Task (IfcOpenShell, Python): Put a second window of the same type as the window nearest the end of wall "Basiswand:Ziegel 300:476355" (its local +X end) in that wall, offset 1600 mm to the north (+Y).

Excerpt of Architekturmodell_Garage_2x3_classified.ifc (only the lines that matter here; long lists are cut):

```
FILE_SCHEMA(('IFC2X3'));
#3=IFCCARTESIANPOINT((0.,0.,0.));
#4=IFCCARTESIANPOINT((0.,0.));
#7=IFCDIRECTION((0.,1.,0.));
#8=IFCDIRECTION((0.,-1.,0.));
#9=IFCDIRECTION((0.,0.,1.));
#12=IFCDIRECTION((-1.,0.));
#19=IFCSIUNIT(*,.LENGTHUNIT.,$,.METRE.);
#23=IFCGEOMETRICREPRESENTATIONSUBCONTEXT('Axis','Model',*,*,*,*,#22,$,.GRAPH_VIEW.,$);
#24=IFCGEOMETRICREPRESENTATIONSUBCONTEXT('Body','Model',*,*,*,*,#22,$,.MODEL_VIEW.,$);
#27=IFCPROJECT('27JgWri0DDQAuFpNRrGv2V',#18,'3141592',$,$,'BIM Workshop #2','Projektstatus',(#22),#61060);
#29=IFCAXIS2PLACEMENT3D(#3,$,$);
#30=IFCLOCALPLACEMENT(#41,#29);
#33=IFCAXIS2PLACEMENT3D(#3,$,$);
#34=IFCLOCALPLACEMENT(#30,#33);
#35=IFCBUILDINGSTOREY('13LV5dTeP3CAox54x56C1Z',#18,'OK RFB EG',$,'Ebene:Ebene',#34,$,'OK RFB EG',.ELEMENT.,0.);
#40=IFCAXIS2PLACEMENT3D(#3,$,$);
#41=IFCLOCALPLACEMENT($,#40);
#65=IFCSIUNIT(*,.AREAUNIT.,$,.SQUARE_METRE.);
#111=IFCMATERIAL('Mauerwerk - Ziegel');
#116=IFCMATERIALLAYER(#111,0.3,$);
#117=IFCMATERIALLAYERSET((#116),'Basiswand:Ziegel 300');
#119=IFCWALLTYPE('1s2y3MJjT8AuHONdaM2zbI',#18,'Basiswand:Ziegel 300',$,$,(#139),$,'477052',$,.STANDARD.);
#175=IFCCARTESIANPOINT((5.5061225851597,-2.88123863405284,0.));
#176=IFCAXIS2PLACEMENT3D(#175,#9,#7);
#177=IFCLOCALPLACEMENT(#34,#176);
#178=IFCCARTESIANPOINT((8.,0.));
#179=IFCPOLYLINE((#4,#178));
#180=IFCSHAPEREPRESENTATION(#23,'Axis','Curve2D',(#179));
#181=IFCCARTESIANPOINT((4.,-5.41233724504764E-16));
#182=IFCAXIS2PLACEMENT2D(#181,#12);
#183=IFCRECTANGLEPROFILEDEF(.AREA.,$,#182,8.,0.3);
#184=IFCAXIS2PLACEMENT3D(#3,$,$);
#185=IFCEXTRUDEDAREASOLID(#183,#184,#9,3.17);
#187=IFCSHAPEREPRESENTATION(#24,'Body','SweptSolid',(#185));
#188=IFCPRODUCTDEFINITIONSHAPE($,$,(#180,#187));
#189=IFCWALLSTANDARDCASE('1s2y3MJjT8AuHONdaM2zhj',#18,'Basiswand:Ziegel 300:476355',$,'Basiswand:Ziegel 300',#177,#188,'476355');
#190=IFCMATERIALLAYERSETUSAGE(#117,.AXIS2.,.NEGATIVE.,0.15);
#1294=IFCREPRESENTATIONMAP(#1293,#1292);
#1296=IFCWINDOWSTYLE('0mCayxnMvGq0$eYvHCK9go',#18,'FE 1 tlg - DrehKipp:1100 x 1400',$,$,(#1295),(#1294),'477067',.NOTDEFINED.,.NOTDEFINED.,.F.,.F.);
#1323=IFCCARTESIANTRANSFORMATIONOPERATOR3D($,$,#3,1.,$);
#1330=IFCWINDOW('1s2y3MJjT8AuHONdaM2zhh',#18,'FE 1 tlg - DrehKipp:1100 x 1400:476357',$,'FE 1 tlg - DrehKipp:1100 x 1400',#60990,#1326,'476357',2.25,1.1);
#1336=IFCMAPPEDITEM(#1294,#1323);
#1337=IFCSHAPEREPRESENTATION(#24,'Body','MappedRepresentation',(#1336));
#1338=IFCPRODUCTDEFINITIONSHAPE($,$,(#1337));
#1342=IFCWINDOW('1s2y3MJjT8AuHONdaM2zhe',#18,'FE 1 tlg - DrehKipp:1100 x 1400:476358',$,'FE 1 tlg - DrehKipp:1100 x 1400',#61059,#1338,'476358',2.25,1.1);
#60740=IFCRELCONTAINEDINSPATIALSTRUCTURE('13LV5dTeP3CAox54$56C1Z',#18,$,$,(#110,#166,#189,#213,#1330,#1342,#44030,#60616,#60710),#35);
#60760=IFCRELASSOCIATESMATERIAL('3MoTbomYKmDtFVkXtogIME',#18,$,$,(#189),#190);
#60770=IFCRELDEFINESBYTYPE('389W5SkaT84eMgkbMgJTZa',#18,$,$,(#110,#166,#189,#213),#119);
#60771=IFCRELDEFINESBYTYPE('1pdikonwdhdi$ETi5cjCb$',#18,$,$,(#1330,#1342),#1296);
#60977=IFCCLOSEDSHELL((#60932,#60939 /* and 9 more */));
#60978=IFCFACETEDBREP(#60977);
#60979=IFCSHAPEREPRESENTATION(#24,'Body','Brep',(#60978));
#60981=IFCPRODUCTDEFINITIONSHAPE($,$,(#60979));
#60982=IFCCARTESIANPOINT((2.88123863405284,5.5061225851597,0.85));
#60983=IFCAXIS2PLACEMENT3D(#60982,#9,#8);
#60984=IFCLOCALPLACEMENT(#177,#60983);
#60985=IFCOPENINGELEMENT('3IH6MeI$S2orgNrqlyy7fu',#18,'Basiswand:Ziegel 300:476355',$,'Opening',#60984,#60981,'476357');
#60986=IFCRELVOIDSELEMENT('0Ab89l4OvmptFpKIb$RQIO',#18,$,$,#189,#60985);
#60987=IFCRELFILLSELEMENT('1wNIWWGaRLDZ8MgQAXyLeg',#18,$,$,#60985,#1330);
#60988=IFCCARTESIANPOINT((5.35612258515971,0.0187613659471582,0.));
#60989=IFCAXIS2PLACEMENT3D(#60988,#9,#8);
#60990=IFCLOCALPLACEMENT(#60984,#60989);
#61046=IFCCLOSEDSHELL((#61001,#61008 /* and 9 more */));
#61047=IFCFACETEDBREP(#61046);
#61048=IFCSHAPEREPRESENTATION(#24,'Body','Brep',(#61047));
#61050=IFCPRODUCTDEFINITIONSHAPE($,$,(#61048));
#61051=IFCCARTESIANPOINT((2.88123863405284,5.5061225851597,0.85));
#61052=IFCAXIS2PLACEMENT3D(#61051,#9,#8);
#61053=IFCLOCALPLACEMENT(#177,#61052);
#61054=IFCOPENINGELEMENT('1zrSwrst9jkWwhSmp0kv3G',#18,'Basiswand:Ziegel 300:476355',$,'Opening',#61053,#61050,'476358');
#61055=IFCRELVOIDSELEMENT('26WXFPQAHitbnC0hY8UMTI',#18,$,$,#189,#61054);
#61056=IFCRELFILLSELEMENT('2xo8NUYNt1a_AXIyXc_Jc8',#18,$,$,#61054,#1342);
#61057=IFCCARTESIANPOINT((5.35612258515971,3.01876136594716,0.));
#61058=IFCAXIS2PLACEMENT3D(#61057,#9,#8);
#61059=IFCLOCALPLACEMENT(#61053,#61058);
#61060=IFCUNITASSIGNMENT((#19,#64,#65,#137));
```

```python
import ifcopenshell
import ifcopenshell.api.feature
import ifcopenshell.api.geometry
import ifcopenshell.api.root
import ifcopenshell.geom
import ifcopenshell.util.element
import ifcopenshell.util.placement
import ifcopenshell.util.shape

model = ifcopenshell.open("Architekturmodell_Garage_2x3_classified.ifc")
settings = ifcopenshell.geom.settings()


def volume(element):
    """Net volume in cubic metres, openings subtracted."""
    shape = ifcopenshell.geom.create_shape(settings, element)
    return ifcopenshell.util.shape.get_volume(shape.geometry)


def reuse_history(source, copy):
    """copy_class also copies each property set's owner history, people and application; keep the originals."""
    for rel in copy.IsDefinedBy:
        if rel.is_a("IfcRelDefinesByProperties") and (history := rel.RelatingPropertyDefinition.OwnerHistory):
            rel.RelatingPropertyDefinition.OwnerHistory = source.OwnerHistory
            ifcopenshell.util.element.remove_deep2(model, history)


window = model.by_guid("1s2y3MJjT8AuHONdaM2zhe")
opening = window.FillsVoids[0].RelatingOpeningElement
wall = opening.VoidsElements[0].RelatingBuildingElement
before = volume(wall)
shift = ifcopenshell.util.placement.get_local_placement(wall.ObjectPlacement)[:3, 0] * 1.6

# copy_class copies the void relationship, type, container and properties, but no geometry.
new_opening = ifcopenshell.api.root.copy_class(model, product=opening)
new_opening.Representation = ifcopenshell.util.element.copy_deep(
    model, opening.Representation, exclude=["IfcGeometricRepresentationContext", "IfcRepresentationMap"]
)
new_opening.Name = "Basiswand:Ziegel 300"
new_opening.Tag = None
new_window = ifcopenshell.api.root.copy_class(model, product=window)
new_window.Representation = ifcopenshell.util.element.copy_deep(
    model, window.Representation, exclude=["IfcGeometricRepresentationContext", "IfcRepresentationMap"]
)
new_window.Name = "FE 1 tlg - DrehKipp:1100 x 1400"
new_window.Tag = None
reuse_history(window, new_window)
fills = ifcopenshell.api.feature.add_filling(model, opening=new_opening, element=new_window)
fills.OwnerHistory = new_window.OwnerHistory  # required in IFC2X3

for old, new in ((opening, new_opening), (window, new_window)):
    matrix = ifcopenshell.util.placement.get_local_placement(old.ObjectPlacement)
    matrix[:3, 3] += shift
    ifcopenshell.api.geometry.edit_object_placement(model, product=new, matrix=matrix, is_si=False)

after = volume(wall)

print(f"wall volume {before:.3f} -> {after:.3f} m3")

model.write("Architekturmodell_Garage_2x3_classified_rev.ifc")
```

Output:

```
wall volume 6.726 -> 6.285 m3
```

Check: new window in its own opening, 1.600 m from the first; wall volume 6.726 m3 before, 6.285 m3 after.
